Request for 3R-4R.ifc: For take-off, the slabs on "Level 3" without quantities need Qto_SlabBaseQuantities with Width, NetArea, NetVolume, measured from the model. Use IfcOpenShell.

First a look at what the model holds.

```python
import ifcopenshell
import ifcopenshell.util.element
import ifcopenshell.util.unit

model = ifcopenshell.open("3R-4R.ifc")
print(model.schema)
for unit_type in ("LENGTHUNIT", "AREAUNIT", "VOLUMEUNIT"):
    print(unit_type, ifcopenshell.util.unit.calculate_unit_scale(model, unit_type))
storey = next(s for s in model.by_type("IfcBuildingStorey") if s.Name == "Level 3")
slabs = [e for e in ifcopenshell.util.element.get_decomposition(storey) if e.is_a("IfcSlab")]
for e in sorted(slabs, key=lambda e: e.id()):
    print(e.id(), e.is_a(), e.Name, list(ifcopenshell.util.element.get_psets(e, qtos_only=True)), sep=" | ")
```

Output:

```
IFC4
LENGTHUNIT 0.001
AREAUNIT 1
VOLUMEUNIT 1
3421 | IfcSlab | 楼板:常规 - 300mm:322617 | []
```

```python
import ifcopenshell
import ifcopenshell.api.pset
import ifcopenshell.geom
import ifcopenshell.util.element
import ifcopenshell.util.shape
import ifcopenshell.util.unit

model = ifcopenshell.open("3R-4R.ifc")
unit_scale = ifcopenshell.util.unit.calculate_unit_scale(model)
area_scale = ifcopenshell.util.unit.calculate_unit_scale(model, "AREAUNIT")
volume_scale = ifcopenshell.util.unit.calculate_unit_scale(model, "VOLUMEUNIT")
settings = ifcopenshell.geom.settings()

storey = next(s for s in model.by_type("IfcBuildingStorey") if s.Name == "Level 3")
slabs = [e for e in ifcopenshell.util.element.get_decomposition(storey) if e.is_a("IfcSlab")]

for e in sorted(slabs, key=lambda e: e.id()):
    if ifcopenshell.util.element.get_psets(e, qtos_only=True, should_inherit=False):
        continue
    # Geometry comes back in metres, in the element's own axes.
    shape = ifcopenshell.geom.create_shape(settings, e)
    values = {
        "Width": ifcopenshell.util.shape.get_z(shape.geometry) / unit_scale,
        "NetArea": ifcopenshell.util.shape.get_footprint_area(shape.geometry) / area_scale,
        "NetVolume": ifcopenshell.util.shape.get_volume(shape.geometry) / volume_scale,
    }
    qto = ifcopenshell.api.pset.add_qto(model, product=e, name="Qto_SlabBaseQuantities")
    ifcopenshell.api.pset.edit_qto(model, qto=qto, properties=values)
    print(e.id(), {k: round(v, 3) for k, v in values.items()})

model.write("3R-4R_rev.ifc")
```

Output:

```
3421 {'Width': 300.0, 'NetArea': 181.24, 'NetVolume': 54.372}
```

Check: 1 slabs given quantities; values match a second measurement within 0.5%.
